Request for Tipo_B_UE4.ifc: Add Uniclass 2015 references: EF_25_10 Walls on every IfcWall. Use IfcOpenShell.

First a look at what the model holds.

```python
import ifcopenshell

model = ifcopenshell.open("Tipo_B_UE4.ifc")
print(model.schema)
print("classifications:", [c.Name for c in model.by_type("IfcClassification")])
for ifc_class in ("IfcDoor", "IfcRoof", "IfcStair", "IfcWall", "IfcWindow"):
    print(ifc_class, len(model.by_type(ifc_class)))
```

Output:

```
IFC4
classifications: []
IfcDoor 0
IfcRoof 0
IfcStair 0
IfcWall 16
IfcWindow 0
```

```python
import ifcopenshell
import ifcopenshell.api.classification

model = ifcopenshell.open("Tipo_B_UE4.ifc")

system = ifcopenshell.api.classification.add_classification(model, classification="Uniclass 2015")

codes = {
    "IfcWall": ("EF_25_10", "Walls"),
}
for ifc_class, (code, name) in codes.items():
    products = model.by_type(ifc_class)
    ifcopenshell.api.classification.add_reference(
        model, products=products, classification=system, identification=code, name=name
    )
    print(code, len(products))

model.write("Tipo_B_UE4-out.ifc")
```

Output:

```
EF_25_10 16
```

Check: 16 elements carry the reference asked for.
